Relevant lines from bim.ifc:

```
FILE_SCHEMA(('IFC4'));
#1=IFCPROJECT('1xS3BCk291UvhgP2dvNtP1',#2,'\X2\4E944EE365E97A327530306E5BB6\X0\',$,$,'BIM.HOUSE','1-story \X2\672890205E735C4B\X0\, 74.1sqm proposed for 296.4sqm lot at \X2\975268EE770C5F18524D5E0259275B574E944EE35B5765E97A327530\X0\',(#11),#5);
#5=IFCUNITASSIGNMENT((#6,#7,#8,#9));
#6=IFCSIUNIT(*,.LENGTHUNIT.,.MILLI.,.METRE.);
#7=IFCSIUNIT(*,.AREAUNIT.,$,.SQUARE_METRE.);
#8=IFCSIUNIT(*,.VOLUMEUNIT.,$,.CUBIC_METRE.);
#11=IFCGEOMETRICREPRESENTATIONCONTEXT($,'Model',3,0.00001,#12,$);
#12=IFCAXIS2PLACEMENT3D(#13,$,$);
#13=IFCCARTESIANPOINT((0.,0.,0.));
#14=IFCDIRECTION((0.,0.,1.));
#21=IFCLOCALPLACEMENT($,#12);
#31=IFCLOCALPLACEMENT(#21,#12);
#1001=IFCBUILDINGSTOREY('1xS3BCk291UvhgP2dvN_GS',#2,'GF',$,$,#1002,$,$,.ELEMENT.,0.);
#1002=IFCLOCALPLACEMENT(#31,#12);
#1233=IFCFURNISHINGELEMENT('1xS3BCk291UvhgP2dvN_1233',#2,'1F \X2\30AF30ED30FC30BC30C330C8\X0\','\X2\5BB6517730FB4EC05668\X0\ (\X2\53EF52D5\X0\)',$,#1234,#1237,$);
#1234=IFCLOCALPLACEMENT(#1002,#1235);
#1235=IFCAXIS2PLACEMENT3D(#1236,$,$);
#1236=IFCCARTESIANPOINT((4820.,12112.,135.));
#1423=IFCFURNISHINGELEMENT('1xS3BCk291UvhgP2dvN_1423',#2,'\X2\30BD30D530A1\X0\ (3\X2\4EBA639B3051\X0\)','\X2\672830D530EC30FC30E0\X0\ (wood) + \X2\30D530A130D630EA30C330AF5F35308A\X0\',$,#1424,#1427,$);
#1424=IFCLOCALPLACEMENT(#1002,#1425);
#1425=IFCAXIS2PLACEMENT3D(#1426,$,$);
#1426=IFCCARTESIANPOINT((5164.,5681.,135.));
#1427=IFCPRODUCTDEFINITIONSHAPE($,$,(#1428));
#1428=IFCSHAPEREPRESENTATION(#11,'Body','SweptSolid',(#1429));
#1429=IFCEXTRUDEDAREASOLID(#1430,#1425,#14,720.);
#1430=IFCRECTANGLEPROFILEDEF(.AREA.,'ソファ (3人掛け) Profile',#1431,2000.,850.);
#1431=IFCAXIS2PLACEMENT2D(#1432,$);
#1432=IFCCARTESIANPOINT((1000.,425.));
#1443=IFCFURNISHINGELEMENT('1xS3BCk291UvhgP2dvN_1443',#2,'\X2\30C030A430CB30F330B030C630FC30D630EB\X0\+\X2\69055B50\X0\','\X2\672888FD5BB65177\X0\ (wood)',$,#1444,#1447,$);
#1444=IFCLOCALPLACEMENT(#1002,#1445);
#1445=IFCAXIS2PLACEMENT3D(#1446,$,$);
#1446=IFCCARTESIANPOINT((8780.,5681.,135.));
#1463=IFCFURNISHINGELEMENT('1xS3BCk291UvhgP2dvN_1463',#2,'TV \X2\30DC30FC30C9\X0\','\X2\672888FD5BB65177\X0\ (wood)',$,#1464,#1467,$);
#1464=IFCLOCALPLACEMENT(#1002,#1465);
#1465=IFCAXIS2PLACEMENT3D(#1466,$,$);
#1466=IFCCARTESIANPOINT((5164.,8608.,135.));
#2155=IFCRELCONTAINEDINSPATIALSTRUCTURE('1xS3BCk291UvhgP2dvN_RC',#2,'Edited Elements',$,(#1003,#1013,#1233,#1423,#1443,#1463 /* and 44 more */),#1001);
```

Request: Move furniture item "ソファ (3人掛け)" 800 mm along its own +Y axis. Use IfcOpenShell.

```python
import ifcopenshell
import ifcopenshell.api.geometry
import ifcopenshell.util.placement
import ifcopenshell.util.unit

model = ifcopenshell.open("bim.ifc")
unit_scale = ifcopenshell.util.unit.calculate_unit_scale(model)

item = model.by_id(1423)
matrix = ifcopenshell.util.placement.get_local_placement(item.ObjectPlacement)
matrix[:3, 3] += matrix[:3, 1] * 0.8 / unit_scale
ifcopenshell.api.geometry.edit_object_placement(model, product=item, matrix=matrix, is_si=False)

print(ifcopenshell.util.placement.get_local_placement(item.ObjectPlacement).round(3) + 0.0)

model.write("bim_rev.ifc")
```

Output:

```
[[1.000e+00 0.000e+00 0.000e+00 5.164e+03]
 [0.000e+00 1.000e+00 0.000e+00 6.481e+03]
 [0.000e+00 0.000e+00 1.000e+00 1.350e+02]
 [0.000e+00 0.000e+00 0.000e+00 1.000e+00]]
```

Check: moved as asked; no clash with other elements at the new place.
